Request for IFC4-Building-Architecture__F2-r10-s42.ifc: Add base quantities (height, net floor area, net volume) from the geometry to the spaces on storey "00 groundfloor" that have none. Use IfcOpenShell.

First a look at what the model holds.

```python
import ifcopenshell
import ifcopenshell.util.element
import ifcopenshell.util.unit

model = ifcopenshell.open("IFC4-Building-Architecture__F2-r10-s42.ifc")
print(model.schema)
for unit_type in ("LENGTHUNIT", "AREAUNIT", "VOLUMEUNIT"):
    print(unit_type, ifcopenshell.util.unit.calculate_unit_scale(model, unit_type))
storey = next(s for s in model.by_type("IfcBuildingStorey") if s.Name == "00 groundfloor")
spaces = [e for e in ifcopenshell.util.element.get_decomposition(storey) if e.is_a("IfcSpace")]
for e in sorted(spaces, key=lambda e: e.id()):
    print(e.id(), e.is_a(), e.Name, list(ifcopenshell.util.element.get_psets(e, qtos_only=True)), sep=" | ")
```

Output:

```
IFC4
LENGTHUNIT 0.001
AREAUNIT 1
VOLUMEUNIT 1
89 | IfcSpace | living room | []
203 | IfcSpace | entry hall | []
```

```python
import ifcopenshell
import ifcopenshell.api.pset
import ifcopenshell.geom
import ifcopenshell.util.element
import ifcopenshell.util.shape
import ifcopenshell.util.unit

model = ifcopenshell.open("IFC4-Building-Architecture__F2-r10-s42.ifc")
unit_scale = ifcopenshell.util.unit.calculate_unit_scale(model)
area_scale = ifcopenshell.util.unit.calculate_unit_scale(model, "AREAUNIT")
volume_scale = ifcopenshell.util.unit.calculate_unit_scale(model, "VOLUMEUNIT")
settings = ifcopenshell.geom.settings()

storey = next(s for s in model.by_type("IfcBuildingStorey") if s.Name == "00 groundfloor")
spaces = [e for e in ifcopenshell.util.element.get_decomposition(storey) if e.is_a("IfcSpace")]

for e in sorted(spaces, key=lambda e: e.id()):
    if ifcopenshell.util.element.get_psets(e, qtos_only=True, should_inherit=False):
        continue
    # Geometry comes back in metres, in the element's own axes.
    shape = ifcopenshell.geom.create_shape(settings, e)
    values = {
        "Height": ifcopenshell.util.shape.get_z(shape.geometry) / unit_scale,
        "NetFloorArea": ifcopenshell.util.shape.get_footprint_area(shape.geometry) / area_scale,
        "NetVolume": ifcopenshell.util.shape.get_volume(shape.geometry) / volume_scale,
    }
    qto = ifcopenshell.api.pset.add_qto(model, product=e, name="Qto_SpaceBaseQuantities")
    ifcopenshell.api.pset.edit_qto(model, qto=qto, properties=values)
    print(e.id(), {k: round(v, 3) for k, v in values.items()})

model.write("IFC4-Building-Architecture__F2-r10-s42-out.ifc")
```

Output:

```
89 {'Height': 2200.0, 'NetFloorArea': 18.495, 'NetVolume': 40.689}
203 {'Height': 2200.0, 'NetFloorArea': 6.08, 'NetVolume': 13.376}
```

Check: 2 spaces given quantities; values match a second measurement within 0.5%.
